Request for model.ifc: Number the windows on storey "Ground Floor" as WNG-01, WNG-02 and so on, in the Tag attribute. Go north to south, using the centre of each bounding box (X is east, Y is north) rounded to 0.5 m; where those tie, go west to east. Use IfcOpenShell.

First a look at what the model holds.

```python
import ifcopenshell
import ifcopenshell.util.element
import ifcopenshell.util.placement

model = ifcopenshell.open("model.ifc")
print(model.schema)
storey = next(s for s in model.by_type("IfcBuildingStorey") if s.Name == "Ground Floor")
windows = [e for e in ifcopenshell.util.element.get_decomposition(storey) if e.is_a("IfcWindow")]
for e in sorted(windows, key=lambda e: e.id()):
    origin = ifcopenshell.util.placement.get_local_placement(e.ObjectPlacement)[:3, 3]
    print(e.id(), e.Tag, e.Name, origin.round(2) + 0.0, sep=" | ")
```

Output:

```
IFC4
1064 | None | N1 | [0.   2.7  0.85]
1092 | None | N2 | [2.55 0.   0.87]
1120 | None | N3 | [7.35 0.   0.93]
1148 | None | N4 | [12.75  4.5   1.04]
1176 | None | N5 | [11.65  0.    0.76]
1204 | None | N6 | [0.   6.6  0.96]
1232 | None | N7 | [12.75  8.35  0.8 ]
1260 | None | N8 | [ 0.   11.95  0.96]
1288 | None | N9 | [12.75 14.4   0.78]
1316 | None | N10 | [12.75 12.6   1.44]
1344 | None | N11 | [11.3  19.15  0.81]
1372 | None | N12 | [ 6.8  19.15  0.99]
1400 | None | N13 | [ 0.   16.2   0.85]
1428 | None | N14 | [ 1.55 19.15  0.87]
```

```python
import ifcopenshell
import ifcopenshell.geom
import ifcopenshell.util.element
import ifcopenshell.util.shape

model = ifcopenshell.open("model.ifc")
settings = ifcopenshell.geom.settings()
settings.set("use-world-coords", True)


def centre(element):
    shape = ifcopenshell.geom.create_shape(settings, element)
    return ifcopenshell.util.shape.get_bbox_centroid(shape.geometry)


storey = next(s for s in model.by_type("IfcBuildingStorey") if s.Name == "Ground Floor")
windows = [e for e in ifcopenshell.util.element.get_decomposition(storey) if e.is_a("IfcWindow")]

# Insertion points can sit at a corner or the storey origin, so sort by the geometry (in metres).
centres = {e: centre(e) for e in windows}
windows.sort(key=lambda e: (-round(centres[e][1] / 0.5), centres[e][0]))

for i, e in enumerate(windows, start=1):
    number = f"WNG-{i:02d}"
    e.Tag = number
    print(e.id(), number)

model.write("model-out.ifc")
```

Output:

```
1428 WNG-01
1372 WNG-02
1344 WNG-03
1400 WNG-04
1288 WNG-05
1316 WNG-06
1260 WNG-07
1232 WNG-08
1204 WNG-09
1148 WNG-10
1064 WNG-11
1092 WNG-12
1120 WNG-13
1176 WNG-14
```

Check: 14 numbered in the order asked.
